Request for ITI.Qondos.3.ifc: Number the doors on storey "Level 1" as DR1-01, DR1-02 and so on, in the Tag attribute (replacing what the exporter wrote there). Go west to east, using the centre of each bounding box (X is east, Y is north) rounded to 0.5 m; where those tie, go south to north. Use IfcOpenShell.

First a look at what the model holds.

```python
import ifcopenshell
import ifcopenshell.util.element
import ifcopenshell.util.placement

model = ifcopenshell.open("ITI.Qondos.3.ifc")
print(model.schema)
storey = next(s for s in model.by_type("IfcBuildingStorey") if s.Name == "Level 1")
doors = [e for e in ifcopenshell.util.element.get_decomposition(storey) if e.is_a("IfcDoor")]
for e in sorted(doors, key=lambda e: e.id()):
    origin = ifcopenshell.util.placement.get_local_placement(e.ObjectPlacement)[:3, 3]
    print(e.id(), e.Tag, e.Name, origin.round(2) + 0.0, sep=" | ")
```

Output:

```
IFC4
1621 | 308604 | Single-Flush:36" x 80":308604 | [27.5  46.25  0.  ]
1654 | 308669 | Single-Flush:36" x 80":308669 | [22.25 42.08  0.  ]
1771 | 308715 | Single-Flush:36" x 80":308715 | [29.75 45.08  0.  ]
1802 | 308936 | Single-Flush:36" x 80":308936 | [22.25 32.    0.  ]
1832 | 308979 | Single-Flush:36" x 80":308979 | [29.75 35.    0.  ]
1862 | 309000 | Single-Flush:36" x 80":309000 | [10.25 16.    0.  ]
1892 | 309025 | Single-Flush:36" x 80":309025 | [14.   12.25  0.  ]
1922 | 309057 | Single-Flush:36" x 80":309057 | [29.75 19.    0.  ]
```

```python
import ifcopenshell
import ifcopenshell.geom
import ifcopenshell.util.element
import ifcopenshell.util.shape

model = ifcopenshell.open("ITI.Qondos.3.ifc")
settings = ifcopenshell.geom.settings()
settings.set("use-world-coords", True)


def centre(element):
    shape = ifcopenshell.geom.create_shape(settings, element)
    return ifcopenshell.util.shape.get_bbox_centroid(shape.geometry)


storey = next(s for s in model.by_type("IfcBuildingStorey") if s.Name == "Level 1")
doors = [e for e in ifcopenshell.util.element.get_decomposition(storey) if e.is_a("IfcDoor")]

# Insertion points can sit at a corner or the storey origin, so sort by the geometry (in metres).
centres = {e: centre(e) for e in doors}
doors.sort(key=lambda e: (round(centres[e][0] / 0.5), centres[e][1]))

for i, e in enumerate(doors, start=1):
    number = f"DR1-{i:02d}"
    e.Tag = number
    print(e.id(), number)

model.write("ITI.Qondos.3_rev.ifc")
```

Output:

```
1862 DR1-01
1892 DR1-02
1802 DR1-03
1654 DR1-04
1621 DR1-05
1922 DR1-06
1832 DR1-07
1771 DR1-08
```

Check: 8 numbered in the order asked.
